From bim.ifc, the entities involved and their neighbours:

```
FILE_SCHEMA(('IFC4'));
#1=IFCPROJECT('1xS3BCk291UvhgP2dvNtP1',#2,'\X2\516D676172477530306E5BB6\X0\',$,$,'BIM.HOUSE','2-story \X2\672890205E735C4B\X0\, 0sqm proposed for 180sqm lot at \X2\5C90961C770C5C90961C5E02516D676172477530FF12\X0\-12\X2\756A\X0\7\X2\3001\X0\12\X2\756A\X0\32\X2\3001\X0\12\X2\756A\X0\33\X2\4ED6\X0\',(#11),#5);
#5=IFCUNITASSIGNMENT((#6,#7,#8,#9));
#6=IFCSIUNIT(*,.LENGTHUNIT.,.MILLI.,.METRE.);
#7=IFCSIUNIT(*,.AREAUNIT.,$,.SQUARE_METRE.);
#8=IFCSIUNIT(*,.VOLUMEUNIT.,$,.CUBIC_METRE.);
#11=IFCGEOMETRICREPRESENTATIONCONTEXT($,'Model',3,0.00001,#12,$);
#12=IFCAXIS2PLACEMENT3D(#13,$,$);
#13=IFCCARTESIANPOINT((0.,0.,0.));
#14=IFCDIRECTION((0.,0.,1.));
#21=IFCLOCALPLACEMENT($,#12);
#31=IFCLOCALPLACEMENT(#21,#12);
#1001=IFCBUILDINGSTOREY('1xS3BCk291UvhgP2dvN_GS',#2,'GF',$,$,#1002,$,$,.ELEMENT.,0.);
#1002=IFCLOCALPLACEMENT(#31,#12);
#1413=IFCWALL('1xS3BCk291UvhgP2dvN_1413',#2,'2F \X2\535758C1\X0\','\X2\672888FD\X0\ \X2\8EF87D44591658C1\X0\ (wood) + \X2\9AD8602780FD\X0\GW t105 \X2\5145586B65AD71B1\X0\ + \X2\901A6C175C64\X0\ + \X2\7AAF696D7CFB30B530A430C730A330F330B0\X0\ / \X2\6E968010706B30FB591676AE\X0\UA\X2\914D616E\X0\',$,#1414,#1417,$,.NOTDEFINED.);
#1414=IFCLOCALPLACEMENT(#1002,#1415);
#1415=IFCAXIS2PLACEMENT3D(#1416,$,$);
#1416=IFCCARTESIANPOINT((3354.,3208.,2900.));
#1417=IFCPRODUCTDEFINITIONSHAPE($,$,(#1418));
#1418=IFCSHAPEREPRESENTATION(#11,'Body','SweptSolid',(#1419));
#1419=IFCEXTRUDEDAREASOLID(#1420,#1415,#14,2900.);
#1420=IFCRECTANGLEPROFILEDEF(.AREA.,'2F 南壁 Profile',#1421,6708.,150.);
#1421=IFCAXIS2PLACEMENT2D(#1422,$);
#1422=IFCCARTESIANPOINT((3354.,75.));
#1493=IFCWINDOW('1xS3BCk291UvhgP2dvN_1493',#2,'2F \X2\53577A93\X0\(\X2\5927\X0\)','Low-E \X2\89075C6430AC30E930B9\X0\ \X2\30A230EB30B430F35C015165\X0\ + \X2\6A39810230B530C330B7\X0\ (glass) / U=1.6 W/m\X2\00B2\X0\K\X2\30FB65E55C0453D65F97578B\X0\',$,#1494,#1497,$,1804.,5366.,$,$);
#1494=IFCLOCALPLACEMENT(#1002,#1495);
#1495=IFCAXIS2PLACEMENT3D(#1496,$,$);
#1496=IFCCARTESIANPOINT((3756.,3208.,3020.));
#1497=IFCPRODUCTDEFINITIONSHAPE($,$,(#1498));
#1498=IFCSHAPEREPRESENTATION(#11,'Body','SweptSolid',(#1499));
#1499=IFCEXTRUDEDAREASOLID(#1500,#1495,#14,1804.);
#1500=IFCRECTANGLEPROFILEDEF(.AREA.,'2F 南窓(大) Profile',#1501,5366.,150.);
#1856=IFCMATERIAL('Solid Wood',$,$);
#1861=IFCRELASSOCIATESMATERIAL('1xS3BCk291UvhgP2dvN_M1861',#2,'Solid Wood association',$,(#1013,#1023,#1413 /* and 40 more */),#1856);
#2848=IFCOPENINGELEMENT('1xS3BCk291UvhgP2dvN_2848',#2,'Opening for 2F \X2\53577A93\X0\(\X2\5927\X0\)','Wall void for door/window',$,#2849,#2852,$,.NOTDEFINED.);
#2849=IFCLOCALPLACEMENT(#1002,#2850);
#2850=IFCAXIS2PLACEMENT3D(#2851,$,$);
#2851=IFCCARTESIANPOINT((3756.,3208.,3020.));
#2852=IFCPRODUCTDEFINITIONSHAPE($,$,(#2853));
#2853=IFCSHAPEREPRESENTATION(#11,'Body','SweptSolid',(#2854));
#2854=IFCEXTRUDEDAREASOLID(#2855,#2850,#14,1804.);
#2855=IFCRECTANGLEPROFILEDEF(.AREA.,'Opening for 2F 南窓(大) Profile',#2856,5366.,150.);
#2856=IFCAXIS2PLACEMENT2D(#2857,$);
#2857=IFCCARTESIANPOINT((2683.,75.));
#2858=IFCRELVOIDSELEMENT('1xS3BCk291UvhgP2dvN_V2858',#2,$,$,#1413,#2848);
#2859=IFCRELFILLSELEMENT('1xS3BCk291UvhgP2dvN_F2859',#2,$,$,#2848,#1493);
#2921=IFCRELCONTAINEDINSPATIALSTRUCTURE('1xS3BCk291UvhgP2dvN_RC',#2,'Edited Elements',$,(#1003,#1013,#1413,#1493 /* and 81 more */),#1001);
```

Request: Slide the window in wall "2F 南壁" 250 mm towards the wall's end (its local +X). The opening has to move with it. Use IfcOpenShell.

```python
import ifcopenshell
import ifcopenshell.api.geometry
import ifcopenshell.util.placement
import ifcopenshell.util.unit

model = ifcopenshell.open("bim.ifc")
unit_scale = ifcopenshell.util.unit.calculate_unit_scale(model)

window = model.by_guid("1xS3BCk291UvhgP2dvN_1493")
opening = window.FillsVoids[0].RelatingOpeningElement
wall = opening.VoidsElements[0].RelatingBuildingElement

wall_matrix = ifcopenshell.util.placement.get_local_placement(wall.ObjectPlacement)
shift = wall_matrix[:3, 0] * 0.25 / unit_scale
before = ifcopenshell.util.placement.get_local_placement(window.ObjectPlacement)[:3, 3].copy()

# The window is not placed relative to its opening, so move both.
for product in (opening, window):
    matrix = ifcopenshell.util.placement.get_local_placement(product.ObjectPlacement)
    matrix[:3, 3] += shift
    ifcopenshell.api.geometry.edit_object_placement(model, product=product, matrix=matrix, is_si=False)

after = ifcopenshell.util.placement.get_local_placement(window.ObjectPlacement)[:3, 3]
print("window moved by", (after - before).round(3) + 0.0)

model.write("bim-out.ifc")
```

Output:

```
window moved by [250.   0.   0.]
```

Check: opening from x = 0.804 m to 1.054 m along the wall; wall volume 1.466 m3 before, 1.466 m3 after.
